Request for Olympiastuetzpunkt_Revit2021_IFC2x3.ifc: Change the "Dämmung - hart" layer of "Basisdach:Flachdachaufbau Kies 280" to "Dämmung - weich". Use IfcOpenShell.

First a look at what the model holds.

```python
import ifcopenshell
import ifcopenshell.util.element

model = ifcopenshell.open("Olympiastuetzpunkt_Revit2021_IFC2x3.ifc")
print(model.schema)
for layer_set in model.by_type("IfcMaterialLayerSet"):
    if layer_set.LayerSetName == "Basisdach:Flachdachaufbau Kies 280":
        for layer in layer_set.MaterialLayers:
            print(layer.id(), layer.Material and layer.Material.Name, layer.LayerThickness, sep=" | ")
        print(len(ifcopenshell.util.element.get_elements_by_material(model, layer_set)), "elements and types use it")
print(sorted(m.Name for m in model.by_type("IfcMaterial") if m.Name)[:60])
```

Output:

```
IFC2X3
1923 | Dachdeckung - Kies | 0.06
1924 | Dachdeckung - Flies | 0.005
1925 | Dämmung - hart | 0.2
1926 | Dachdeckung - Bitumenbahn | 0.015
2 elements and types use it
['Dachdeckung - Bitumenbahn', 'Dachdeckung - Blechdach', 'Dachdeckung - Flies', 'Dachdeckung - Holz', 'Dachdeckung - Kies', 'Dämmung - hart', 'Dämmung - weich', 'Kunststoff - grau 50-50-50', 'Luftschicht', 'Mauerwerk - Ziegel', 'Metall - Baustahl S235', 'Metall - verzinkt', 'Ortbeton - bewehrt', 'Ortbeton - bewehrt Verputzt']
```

```python
import ifcopenshell
import ifcopenshell.api.material

model = ifcopenshell.open("Olympiastuetzpunkt_Revit2021_IFC2x3.ifc")

layer_set = next(s for s in model.by_type("IfcMaterialLayerSet") if s.LayerSetName == "Basisdach:Flachdachaufbau Kies 280")
layer = next(l for l in layer_set.MaterialLayers if l.Material and l.Material.Name == "Dämmung - hart")
material = next(m for m in model.by_type("IfcMaterial") if m.Name == "Dämmung - weich")

# Point this one layer at the other material; renaming the old one would change it everywhere.
ifcopenshell.api.material.edit_layer(model, layer=layer, attributes={}, material=material)

print([l.Material.Name if l.Material else None for l in layer_set.MaterialLayers])

model.write("Olympiastuetzpunkt_Revit2021_IFC2x3_updated.ifc")
```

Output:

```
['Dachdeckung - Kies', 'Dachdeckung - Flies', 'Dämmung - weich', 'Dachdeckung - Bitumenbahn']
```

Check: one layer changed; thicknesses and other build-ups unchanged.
